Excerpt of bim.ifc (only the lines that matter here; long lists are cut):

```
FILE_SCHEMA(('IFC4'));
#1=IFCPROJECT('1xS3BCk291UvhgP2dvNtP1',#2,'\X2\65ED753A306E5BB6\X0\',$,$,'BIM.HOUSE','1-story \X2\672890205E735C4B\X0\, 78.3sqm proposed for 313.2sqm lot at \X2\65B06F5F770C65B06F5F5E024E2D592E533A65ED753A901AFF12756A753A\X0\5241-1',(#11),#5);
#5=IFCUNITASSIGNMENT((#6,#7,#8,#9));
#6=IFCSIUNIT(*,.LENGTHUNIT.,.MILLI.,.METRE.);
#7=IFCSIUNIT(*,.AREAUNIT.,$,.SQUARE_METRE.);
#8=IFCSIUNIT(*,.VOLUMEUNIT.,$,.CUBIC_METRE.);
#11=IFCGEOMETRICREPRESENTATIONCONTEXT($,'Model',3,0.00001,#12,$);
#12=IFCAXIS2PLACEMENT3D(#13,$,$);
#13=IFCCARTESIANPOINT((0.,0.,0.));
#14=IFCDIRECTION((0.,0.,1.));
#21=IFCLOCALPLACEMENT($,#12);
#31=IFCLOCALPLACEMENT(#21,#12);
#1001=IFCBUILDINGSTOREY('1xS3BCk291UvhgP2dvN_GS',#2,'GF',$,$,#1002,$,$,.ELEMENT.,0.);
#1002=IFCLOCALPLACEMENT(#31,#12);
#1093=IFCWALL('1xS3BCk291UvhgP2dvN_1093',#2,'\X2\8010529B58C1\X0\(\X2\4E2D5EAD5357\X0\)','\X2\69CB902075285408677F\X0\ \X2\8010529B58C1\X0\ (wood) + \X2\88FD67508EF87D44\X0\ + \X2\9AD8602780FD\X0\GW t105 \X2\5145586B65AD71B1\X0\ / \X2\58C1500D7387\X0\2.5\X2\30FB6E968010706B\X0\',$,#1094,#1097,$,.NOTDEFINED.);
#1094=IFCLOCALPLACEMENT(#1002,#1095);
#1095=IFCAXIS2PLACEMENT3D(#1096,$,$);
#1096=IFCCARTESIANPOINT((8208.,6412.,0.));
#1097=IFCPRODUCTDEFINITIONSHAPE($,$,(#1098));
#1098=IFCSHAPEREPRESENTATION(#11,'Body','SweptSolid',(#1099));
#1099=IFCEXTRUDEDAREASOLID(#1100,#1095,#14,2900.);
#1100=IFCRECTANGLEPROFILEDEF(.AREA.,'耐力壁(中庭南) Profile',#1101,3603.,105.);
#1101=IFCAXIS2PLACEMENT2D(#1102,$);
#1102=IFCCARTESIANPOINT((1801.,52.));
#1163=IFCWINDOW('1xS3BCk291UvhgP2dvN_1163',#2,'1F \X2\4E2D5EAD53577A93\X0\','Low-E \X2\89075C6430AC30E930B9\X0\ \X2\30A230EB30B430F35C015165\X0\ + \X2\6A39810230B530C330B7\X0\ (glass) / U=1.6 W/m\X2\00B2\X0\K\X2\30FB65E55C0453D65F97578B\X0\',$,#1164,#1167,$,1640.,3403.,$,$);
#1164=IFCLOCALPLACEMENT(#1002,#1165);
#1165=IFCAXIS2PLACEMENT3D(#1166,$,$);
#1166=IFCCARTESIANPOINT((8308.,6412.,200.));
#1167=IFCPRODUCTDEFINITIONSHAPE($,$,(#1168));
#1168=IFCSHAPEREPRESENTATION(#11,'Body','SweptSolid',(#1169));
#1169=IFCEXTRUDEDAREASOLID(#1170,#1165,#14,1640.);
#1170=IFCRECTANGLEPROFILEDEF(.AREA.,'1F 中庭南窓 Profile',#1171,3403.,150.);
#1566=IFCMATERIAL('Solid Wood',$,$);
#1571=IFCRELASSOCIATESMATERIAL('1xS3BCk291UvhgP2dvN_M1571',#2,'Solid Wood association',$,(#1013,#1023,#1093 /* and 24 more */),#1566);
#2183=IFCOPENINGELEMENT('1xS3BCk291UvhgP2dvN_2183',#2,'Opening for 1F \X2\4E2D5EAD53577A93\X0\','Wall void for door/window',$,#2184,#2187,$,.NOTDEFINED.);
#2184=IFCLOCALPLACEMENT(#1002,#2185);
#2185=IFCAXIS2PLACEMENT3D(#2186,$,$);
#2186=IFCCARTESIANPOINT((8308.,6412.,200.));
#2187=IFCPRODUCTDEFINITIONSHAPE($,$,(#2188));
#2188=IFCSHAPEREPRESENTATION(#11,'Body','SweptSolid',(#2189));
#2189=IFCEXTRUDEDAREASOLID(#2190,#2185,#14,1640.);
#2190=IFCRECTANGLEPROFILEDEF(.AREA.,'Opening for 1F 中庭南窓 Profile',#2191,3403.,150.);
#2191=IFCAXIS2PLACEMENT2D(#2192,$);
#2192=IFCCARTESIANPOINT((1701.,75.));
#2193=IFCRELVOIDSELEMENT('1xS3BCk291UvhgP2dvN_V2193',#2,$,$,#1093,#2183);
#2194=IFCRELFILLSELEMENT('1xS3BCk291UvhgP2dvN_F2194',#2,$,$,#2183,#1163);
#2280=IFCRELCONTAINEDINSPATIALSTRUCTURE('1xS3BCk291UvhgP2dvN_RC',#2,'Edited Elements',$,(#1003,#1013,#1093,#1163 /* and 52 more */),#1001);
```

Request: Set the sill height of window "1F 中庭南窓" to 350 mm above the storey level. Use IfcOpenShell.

```python
import numpy as np
import ifcopenshell
import ifcopenshell.api.geometry
import ifcopenshell.geom
import ifcopenshell.util.element
import ifcopenshell.util.placement
import ifcopenshell.util.shape
import ifcopenshell.util.unit

model = ifcopenshell.open("bim.ifc")
unit_scale = ifcopenshell.util.unit.calculate_unit_scale(model)

window = model.by_guid("1xS3BCk291UvhgP2dvN_1163")
opening = window.FillsVoids[0].RelatingOpeningElement
storey = ifcopenshell.util.element.get_container(window, ifc_class="IfcBuildingStorey")
level = ifcopenshell.util.placement.get_local_placement(storey.ObjectPlacement)[2, 3]

# The opening's origin need not be at the sill, so measure its lowest point.
shape = ifcopenshell.geom.create_shape(ifcopenshell.geom.settings(), opening)
bottom = ifcopenshell.util.shape.get_shape_bottom_elevation(shape, shape.geometry) / unit_scale
dz = level + 0.35 / unit_scale - bottom

shift = np.array([0.0, 0.0, dz])
# The window is not placed relative to its opening, so move both.
for product in (opening, window):
    matrix = ifcopenshell.util.placement.get_local_placement(product.ObjectPlacement)
    matrix[:3, 3] += shift
    ifcopenshell.api.geometry.edit_object_placement(model, product=product, matrix=matrix, is_si=False)

print(f"moved by {dz * unit_scale:+.3f} m")

model.write("bim_edited.ifc")
```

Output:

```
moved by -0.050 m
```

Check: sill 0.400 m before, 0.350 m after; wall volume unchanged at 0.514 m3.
